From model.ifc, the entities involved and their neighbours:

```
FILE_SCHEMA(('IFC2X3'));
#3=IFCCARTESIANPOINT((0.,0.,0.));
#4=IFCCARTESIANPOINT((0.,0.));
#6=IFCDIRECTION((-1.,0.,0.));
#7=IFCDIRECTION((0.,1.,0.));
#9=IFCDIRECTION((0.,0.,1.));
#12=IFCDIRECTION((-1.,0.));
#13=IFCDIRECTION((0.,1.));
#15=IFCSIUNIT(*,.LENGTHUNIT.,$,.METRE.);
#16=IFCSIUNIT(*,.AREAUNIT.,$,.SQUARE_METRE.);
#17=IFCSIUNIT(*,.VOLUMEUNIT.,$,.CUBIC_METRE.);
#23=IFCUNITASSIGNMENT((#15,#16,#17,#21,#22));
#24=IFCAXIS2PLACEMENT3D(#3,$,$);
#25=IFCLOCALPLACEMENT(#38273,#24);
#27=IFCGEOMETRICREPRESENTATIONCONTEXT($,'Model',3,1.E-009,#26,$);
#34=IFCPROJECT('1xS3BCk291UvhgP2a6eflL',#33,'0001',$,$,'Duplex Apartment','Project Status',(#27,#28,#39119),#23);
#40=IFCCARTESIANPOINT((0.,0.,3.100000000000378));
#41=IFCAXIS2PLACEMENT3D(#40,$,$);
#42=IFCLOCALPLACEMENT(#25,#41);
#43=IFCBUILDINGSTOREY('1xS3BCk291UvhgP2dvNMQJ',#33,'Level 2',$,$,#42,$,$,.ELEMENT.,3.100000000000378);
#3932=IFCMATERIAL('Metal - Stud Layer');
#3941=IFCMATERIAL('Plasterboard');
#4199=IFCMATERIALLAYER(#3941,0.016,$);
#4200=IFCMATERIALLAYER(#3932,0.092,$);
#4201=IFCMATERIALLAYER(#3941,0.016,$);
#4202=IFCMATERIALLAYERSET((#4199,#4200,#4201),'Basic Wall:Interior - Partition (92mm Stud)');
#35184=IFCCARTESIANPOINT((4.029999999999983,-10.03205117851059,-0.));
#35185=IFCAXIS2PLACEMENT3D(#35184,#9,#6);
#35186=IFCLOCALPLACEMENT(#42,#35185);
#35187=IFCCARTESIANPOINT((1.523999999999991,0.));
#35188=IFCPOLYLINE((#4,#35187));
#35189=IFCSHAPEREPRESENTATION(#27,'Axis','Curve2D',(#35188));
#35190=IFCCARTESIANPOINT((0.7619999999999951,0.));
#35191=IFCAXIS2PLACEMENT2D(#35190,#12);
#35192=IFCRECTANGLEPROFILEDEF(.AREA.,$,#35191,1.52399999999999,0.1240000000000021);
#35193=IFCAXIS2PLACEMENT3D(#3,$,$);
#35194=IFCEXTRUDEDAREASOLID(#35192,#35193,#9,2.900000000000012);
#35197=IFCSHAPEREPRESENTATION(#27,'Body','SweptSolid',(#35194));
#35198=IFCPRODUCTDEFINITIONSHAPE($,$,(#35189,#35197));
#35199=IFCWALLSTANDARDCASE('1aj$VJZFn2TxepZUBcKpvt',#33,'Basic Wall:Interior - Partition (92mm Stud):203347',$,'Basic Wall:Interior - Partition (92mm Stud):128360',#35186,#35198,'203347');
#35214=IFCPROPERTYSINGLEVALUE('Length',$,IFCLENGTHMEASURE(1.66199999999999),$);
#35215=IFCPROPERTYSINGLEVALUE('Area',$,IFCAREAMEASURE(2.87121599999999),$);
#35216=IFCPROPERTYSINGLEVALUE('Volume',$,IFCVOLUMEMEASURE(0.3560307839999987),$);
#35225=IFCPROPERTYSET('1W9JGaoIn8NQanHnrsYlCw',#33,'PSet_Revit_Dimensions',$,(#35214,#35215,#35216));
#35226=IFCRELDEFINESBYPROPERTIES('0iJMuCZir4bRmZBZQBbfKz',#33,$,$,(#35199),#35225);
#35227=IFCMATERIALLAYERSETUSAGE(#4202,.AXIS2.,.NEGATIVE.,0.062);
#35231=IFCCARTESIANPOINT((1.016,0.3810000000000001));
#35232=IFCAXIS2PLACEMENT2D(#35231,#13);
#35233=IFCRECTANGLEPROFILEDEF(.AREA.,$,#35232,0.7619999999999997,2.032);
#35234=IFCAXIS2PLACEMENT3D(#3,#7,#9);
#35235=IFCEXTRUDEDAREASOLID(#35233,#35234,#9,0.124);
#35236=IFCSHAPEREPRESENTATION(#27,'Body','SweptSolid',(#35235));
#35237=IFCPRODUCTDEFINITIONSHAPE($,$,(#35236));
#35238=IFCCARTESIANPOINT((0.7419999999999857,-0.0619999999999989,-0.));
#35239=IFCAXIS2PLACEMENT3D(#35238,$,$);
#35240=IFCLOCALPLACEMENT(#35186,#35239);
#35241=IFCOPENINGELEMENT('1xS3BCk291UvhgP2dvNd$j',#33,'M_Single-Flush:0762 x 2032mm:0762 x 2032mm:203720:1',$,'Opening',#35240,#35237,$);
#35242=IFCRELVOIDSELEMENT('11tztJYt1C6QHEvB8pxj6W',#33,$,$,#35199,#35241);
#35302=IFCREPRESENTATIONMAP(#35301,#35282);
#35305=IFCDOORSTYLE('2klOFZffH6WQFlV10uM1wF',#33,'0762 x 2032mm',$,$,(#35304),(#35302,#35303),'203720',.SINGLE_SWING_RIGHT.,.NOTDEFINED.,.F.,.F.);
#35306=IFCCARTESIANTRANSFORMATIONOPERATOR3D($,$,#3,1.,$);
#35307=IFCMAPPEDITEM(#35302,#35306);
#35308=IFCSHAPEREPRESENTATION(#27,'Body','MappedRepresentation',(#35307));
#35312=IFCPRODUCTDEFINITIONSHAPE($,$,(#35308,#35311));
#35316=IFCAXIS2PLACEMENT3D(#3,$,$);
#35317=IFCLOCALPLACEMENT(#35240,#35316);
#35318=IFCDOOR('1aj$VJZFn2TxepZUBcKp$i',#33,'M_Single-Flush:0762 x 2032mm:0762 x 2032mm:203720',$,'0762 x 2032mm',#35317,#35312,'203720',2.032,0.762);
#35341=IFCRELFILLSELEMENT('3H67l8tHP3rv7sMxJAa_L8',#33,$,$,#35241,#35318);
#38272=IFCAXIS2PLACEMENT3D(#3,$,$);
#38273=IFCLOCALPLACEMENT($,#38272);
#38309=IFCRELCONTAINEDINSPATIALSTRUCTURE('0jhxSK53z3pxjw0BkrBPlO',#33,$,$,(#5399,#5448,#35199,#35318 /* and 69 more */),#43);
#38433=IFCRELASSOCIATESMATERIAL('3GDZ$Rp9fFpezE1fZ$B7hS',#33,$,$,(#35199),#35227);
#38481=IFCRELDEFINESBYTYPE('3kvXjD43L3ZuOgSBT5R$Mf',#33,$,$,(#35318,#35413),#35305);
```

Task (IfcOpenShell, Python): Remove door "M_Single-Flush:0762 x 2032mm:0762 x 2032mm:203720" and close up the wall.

```python
import ifcopenshell
import ifcopenshell.api.feature
import ifcopenshell.api.pset
import ifcopenshell.api.root
import ifcopenshell.geom
import ifcopenshell.util.element
import ifcopenshell.util.shape
import ifcopenshell.util.unit

model = ifcopenshell.open("model.ifc")
area_scale = ifcopenshell.util.unit.calculate_unit_scale(model, "AREAUNIT")
volume_scale = ifcopenshell.util.unit.calculate_unit_scale(model, "VOLUMEUNIT")
settings = ifcopenshell.geom.settings()


def volume(element):
    """Net volume in cubic metres, openings subtracted."""
    shape = ifcopenshell.geom.create_shape(settings, element)
    return ifcopenshell.util.shape.get_volume(shape.geometry)


door = model.by_guid("1aj$VJZFn2TxepZUBcKp$i")
opening = door.FillsVoids[0].RelatingOpeningElement
wall = opening.VoidsElements[0].RelatingBuildingElement
before = volume(wall)

ifcopenshell.api.root.remove_product(model, product=door)
ifcopenshell.api.feature.remove_feature(model, feature=opening)

after = volume(wall)
thickness = 0.124  # wall thickness in metres

# Update the wall's stored quantities.
pset = model.by_id(ifcopenshell.util.element.get_pset(wall, "PSet_Revit_Dimensions", should_inherit=False)["id"])
ifcopenshell.api.pset.edit_pset(model, pset=pset, properties={
    "Area": model.create_entity("IfcAreaMeasure", after / thickness / area_scale),
    "Volume": model.create_entity("IfcVolumeMeasure", after / volume_scale),
})

print(f"wall volume {before:.3f} -> {after:.3f} m3")

model.write("model_v2.ifc")
```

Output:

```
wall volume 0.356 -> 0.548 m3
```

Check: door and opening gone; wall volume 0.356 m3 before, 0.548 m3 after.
